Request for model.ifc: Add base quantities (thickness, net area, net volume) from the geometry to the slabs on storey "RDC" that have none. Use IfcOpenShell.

First a look at what the model holds.

```python
import ifcopenshell
import ifcopenshell.util.element
import ifcopenshell.util.unit

model = ifcopenshell.open("model.ifc")
print(model.schema)
for unit_type in ("LENGTHUNIT", "AREAUNIT", "VOLUMEUNIT"):
    print(unit_type, ifcopenshell.util.unit.calculate_unit_scale(model, unit_type))
storey = next(s for s in model.by_type("IfcBuildingStorey") if s.Name == "RDC")
slabs = [e for e in ifcopenshell.util.element.get_decomposition(storey) if e.is_a("IfcSlab")]
for e in sorted(slabs, key=lambda e: e.id()):
    print(e.id(), e.is_a(), e.Name, list(ifcopenshell.util.element.get_psets(e, qtos_only=True)), sep=" | ")
```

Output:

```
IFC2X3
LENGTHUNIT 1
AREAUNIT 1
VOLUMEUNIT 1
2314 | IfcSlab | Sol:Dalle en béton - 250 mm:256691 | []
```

```python
import ifcopenshell
import ifcopenshell.api.pset
import ifcopenshell.geom
import ifcopenshell.util.element
import ifcopenshell.util.shape
import ifcopenshell.util.unit

model = ifcopenshell.open("model.ifc")
unit_scale = ifcopenshell.util.unit.calculate_unit_scale(model)
area_scale = ifcopenshell.util.unit.calculate_unit_scale(model, "AREAUNIT")
volume_scale = ifcopenshell.util.unit.calculate_unit_scale(model, "VOLUMEUNIT")
settings = ifcopenshell.geom.settings()

storey = next(s for s in model.by_type("IfcBuildingStorey") if s.Name == "RDC")
slabs = [e for e in ifcopenshell.util.element.get_decomposition(storey) if e.is_a("IfcSlab")]

for e in sorted(slabs, key=lambda e: e.id()):
    if ifcopenshell.util.element.get_psets(e, qtos_only=True, should_inherit=False):
        continue
    # Geometry comes back in metres, in the element's own axes.
    shape = ifcopenshell.geom.create_shape(settings, e)
    values = {
        "Width": ifcopenshell.util.shape.get_z(shape.geometry) / unit_scale,
        "NetArea": ifcopenshell.util.shape.get_footprint_area(shape.geometry) / area_scale,
        "NetVolume": ifcopenshell.util.shape.get_volume(shape.geometry) / volume_scale,
    }
    qto = ifcopenshell.api.pset.add_qto(model, product=e, name="BaseQuantities")
    ifcopenshell.api.pset.edit_qto(model, qto=qto, properties=values)
    print(e.id(), {k: round(v, 3) for k, v in values.items()})

model.write("model_rev.ifc")
```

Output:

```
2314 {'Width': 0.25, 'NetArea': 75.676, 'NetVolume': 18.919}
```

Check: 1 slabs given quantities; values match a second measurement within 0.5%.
